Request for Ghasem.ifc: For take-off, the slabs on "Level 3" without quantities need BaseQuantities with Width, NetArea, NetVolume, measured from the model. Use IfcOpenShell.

First a look at what the model holds.

```python
import ifcopenshell
import ifcopenshell.util.element
import ifcopenshell.util.unit

model = ifcopenshell.open("Ghasem.ifc")
print(model.schema)
for unit_type in ("LENGTHUNIT", "AREAUNIT", "VOLUMEUNIT"):
    print(unit_type, ifcopenshell.util.unit.calculate_unit_scale(model, unit_type))
storey = next(s for s in model.by_type("IfcBuildingStorey") if s.Name == "Level 3")
slabs = [e for e in ifcopenshell.util.element.get_decomposition(storey) if e.is_a("IfcSlab")]
for e in sorted(slabs, key=lambda e: e.id()):
    print(e.id(), e.is_a(), e.Name, list(ifcopenshell.util.element.get_psets(e, qtos_only=True)), sep=" | ")
```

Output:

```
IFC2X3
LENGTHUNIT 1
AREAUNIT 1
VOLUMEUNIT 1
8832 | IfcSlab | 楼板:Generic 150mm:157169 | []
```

```python
import ifcopenshell
import ifcopenshell.api.pset
import ifcopenshell.geom
import ifcopenshell.util.element
import ifcopenshell.util.shape
import ifcopenshell.util.unit

model = ifcopenshell.open("Ghasem.ifc")
unit_scale = ifcopenshell.util.unit.calculate_unit_scale(model)
area_scale = ifcopenshell.util.unit.calculate_unit_scale(model, "AREAUNIT")
volume_scale = ifcopenshell.util.unit.calculate_unit_scale(model, "VOLUMEUNIT")
settings = ifcopenshell.geom.settings()

storey = next(s for s in model.by_type("IfcBuildingStorey") if s.Name == "Level 3")
slabs = [e for e in ifcopenshell.util.element.get_decomposition(storey) if e.is_a("IfcSlab")]

for e in sorted(slabs, key=lambda e: e.id()):
    if ifcopenshell.util.element.get_psets(e, qtos_only=True, should_inherit=False):
        continue
    # Geometry comes back in metres, in the element's own axes.
    shape = ifcopenshell.geom.create_shape(settings, e)
    values = {
        "Width": ifcopenshell.util.shape.get_z(shape.geometry) / unit_scale,
        "NetArea": ifcopenshell.util.shape.get_footprint_area(shape.geometry) / area_scale,
        "NetVolume": ifcopenshell.util.shape.get_volume(shape.geometry) / volume_scale,
    }
    qto = ifcopenshell.api.pset.add_qto(model, product=e, name="BaseQuantities")
    ifcopenshell.api.pset.edit_qto(model, qto=qto, properties=values)
    print(e.id(), {k: round(v, 3) for k, v in values.items()})

model.write("Ghasem_rev.ifc")
```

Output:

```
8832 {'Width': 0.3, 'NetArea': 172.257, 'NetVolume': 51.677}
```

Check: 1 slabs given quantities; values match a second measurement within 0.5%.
